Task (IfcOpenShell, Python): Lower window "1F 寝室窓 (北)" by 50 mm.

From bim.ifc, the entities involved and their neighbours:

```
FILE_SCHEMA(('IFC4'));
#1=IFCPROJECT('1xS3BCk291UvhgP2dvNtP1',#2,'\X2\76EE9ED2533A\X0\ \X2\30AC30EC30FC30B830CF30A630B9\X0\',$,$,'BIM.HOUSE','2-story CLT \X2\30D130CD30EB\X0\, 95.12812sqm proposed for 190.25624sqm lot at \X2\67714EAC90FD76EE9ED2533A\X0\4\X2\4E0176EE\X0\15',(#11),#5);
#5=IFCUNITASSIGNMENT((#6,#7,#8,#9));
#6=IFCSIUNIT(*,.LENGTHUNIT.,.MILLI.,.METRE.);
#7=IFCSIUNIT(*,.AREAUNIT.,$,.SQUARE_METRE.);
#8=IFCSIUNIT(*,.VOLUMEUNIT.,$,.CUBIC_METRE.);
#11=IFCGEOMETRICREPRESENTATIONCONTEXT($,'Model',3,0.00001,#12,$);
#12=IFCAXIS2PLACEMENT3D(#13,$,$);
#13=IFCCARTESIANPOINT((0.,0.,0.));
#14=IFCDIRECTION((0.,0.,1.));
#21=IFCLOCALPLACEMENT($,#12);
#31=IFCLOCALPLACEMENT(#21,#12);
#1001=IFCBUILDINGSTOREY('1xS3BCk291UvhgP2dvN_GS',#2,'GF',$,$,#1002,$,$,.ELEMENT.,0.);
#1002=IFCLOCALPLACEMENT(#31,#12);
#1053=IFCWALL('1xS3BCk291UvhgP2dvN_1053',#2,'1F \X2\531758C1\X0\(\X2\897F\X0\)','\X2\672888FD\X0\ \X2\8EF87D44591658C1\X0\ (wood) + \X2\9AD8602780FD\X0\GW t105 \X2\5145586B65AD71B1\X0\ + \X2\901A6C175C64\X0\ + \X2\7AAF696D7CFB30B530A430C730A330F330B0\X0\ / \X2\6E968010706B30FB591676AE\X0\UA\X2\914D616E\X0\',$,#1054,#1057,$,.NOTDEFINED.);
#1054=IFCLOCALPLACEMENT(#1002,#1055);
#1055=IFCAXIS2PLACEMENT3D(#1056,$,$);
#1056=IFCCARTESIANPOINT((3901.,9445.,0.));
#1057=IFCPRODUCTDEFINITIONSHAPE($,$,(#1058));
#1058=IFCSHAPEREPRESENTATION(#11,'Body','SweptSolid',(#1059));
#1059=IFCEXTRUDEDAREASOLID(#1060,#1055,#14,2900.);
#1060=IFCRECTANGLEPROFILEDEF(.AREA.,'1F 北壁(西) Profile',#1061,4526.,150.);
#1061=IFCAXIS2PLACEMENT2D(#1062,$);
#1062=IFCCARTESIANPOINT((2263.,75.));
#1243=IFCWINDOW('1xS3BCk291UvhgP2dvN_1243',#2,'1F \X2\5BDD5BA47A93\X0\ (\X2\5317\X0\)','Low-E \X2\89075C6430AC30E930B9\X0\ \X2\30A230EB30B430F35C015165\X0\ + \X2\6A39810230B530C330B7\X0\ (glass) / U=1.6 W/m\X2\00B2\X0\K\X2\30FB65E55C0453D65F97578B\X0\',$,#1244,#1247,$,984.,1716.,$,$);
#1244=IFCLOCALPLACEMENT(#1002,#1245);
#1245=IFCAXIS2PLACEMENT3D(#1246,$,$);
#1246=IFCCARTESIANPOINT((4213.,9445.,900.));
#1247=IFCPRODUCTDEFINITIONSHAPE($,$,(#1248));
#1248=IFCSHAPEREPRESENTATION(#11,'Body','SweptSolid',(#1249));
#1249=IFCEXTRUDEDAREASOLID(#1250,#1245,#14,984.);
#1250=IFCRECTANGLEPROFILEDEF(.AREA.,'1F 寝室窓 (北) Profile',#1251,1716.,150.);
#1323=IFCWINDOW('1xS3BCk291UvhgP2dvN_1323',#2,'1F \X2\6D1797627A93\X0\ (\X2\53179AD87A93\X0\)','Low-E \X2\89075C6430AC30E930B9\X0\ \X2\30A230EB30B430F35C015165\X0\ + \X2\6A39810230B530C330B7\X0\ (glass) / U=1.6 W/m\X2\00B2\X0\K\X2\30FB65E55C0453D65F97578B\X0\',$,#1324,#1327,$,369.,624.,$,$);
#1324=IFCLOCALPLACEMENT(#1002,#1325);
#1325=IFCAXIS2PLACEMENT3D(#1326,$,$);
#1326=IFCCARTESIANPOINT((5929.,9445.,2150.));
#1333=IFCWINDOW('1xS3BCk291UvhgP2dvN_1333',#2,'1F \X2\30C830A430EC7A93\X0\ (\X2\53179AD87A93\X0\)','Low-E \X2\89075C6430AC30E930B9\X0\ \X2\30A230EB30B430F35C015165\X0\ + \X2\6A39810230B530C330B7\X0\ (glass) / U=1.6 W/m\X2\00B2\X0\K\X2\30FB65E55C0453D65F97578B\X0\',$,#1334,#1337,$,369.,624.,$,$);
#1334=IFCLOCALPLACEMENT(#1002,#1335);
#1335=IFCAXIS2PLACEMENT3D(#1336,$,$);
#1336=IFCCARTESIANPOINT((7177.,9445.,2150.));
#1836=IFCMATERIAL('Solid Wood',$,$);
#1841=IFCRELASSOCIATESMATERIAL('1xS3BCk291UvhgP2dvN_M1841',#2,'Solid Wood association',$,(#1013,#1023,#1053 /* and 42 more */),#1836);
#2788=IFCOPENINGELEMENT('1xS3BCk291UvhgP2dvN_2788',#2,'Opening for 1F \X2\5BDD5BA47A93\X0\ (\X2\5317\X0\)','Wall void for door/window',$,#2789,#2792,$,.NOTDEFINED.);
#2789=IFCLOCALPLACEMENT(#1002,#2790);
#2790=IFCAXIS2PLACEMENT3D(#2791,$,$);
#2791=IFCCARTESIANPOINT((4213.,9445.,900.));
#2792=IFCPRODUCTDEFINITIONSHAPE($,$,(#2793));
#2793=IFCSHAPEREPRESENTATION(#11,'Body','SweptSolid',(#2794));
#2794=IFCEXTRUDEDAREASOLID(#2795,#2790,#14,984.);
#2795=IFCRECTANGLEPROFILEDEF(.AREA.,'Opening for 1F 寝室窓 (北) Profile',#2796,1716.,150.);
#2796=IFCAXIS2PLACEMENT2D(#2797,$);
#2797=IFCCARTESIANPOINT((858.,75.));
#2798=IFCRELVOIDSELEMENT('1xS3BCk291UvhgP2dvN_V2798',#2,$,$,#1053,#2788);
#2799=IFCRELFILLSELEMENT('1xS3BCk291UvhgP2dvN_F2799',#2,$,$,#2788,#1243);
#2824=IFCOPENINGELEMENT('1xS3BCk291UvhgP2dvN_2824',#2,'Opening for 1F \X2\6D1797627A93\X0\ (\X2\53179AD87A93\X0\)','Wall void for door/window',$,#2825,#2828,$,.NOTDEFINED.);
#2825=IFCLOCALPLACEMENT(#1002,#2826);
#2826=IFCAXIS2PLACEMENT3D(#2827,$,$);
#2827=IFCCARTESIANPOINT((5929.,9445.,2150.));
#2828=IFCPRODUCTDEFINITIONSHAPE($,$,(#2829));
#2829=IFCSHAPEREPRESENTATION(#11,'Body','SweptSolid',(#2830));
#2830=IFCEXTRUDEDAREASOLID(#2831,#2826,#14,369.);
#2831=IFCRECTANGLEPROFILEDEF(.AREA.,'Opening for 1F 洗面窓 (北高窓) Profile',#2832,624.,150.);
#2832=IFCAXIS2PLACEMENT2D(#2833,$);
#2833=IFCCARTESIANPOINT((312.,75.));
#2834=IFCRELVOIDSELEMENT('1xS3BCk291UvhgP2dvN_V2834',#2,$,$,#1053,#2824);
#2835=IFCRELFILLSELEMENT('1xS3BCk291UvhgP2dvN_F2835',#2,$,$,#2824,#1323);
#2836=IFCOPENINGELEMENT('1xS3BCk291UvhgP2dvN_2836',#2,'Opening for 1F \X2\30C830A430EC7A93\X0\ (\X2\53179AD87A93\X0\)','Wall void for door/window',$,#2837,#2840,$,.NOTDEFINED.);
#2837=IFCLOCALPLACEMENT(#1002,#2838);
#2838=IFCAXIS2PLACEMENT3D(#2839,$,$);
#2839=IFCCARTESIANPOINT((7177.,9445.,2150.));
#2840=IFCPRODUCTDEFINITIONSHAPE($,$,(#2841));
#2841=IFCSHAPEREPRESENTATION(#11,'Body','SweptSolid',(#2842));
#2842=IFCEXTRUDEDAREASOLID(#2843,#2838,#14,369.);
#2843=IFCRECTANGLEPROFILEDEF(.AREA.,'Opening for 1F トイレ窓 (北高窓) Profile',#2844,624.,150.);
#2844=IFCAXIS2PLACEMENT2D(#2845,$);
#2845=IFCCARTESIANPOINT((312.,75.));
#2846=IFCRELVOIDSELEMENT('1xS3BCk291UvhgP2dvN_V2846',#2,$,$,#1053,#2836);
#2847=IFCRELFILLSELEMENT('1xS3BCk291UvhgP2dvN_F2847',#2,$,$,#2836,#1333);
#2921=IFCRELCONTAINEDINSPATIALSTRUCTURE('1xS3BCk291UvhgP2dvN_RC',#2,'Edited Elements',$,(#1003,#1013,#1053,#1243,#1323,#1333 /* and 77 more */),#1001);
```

```python
import numpy as np
import ifcopenshell
import ifcopenshell.api.geometry
import ifcopenshell.util.placement
import ifcopenshell.util.unit

model = ifcopenshell.open("bim.ifc")
unit_scale = ifcopenshell.util.unit.calculate_unit_scale(model)

window = model.by_guid("1xS3BCk291UvhgP2dvN_1243")
opening = window.FillsVoids[0].RelatingOpeningElement
dz = -0.05 / unit_scale

shift = np.array([0.0, 0.0, dz])
# The window is not placed relative to its opening, so move both.
for product in (opening, window):
    matrix = ifcopenshell.util.placement.get_local_placement(product.ObjectPlacement)
    matrix[:3, 3] += shift
    ifcopenshell.api.geometry.edit_object_placement(model, product=product, matrix=matrix, is_si=False)

print(f"moved by {dz * unit_scale:+.3f} m")

model.write("bim_rev.ifc")
```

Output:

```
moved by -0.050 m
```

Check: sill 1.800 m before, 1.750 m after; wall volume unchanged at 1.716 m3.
